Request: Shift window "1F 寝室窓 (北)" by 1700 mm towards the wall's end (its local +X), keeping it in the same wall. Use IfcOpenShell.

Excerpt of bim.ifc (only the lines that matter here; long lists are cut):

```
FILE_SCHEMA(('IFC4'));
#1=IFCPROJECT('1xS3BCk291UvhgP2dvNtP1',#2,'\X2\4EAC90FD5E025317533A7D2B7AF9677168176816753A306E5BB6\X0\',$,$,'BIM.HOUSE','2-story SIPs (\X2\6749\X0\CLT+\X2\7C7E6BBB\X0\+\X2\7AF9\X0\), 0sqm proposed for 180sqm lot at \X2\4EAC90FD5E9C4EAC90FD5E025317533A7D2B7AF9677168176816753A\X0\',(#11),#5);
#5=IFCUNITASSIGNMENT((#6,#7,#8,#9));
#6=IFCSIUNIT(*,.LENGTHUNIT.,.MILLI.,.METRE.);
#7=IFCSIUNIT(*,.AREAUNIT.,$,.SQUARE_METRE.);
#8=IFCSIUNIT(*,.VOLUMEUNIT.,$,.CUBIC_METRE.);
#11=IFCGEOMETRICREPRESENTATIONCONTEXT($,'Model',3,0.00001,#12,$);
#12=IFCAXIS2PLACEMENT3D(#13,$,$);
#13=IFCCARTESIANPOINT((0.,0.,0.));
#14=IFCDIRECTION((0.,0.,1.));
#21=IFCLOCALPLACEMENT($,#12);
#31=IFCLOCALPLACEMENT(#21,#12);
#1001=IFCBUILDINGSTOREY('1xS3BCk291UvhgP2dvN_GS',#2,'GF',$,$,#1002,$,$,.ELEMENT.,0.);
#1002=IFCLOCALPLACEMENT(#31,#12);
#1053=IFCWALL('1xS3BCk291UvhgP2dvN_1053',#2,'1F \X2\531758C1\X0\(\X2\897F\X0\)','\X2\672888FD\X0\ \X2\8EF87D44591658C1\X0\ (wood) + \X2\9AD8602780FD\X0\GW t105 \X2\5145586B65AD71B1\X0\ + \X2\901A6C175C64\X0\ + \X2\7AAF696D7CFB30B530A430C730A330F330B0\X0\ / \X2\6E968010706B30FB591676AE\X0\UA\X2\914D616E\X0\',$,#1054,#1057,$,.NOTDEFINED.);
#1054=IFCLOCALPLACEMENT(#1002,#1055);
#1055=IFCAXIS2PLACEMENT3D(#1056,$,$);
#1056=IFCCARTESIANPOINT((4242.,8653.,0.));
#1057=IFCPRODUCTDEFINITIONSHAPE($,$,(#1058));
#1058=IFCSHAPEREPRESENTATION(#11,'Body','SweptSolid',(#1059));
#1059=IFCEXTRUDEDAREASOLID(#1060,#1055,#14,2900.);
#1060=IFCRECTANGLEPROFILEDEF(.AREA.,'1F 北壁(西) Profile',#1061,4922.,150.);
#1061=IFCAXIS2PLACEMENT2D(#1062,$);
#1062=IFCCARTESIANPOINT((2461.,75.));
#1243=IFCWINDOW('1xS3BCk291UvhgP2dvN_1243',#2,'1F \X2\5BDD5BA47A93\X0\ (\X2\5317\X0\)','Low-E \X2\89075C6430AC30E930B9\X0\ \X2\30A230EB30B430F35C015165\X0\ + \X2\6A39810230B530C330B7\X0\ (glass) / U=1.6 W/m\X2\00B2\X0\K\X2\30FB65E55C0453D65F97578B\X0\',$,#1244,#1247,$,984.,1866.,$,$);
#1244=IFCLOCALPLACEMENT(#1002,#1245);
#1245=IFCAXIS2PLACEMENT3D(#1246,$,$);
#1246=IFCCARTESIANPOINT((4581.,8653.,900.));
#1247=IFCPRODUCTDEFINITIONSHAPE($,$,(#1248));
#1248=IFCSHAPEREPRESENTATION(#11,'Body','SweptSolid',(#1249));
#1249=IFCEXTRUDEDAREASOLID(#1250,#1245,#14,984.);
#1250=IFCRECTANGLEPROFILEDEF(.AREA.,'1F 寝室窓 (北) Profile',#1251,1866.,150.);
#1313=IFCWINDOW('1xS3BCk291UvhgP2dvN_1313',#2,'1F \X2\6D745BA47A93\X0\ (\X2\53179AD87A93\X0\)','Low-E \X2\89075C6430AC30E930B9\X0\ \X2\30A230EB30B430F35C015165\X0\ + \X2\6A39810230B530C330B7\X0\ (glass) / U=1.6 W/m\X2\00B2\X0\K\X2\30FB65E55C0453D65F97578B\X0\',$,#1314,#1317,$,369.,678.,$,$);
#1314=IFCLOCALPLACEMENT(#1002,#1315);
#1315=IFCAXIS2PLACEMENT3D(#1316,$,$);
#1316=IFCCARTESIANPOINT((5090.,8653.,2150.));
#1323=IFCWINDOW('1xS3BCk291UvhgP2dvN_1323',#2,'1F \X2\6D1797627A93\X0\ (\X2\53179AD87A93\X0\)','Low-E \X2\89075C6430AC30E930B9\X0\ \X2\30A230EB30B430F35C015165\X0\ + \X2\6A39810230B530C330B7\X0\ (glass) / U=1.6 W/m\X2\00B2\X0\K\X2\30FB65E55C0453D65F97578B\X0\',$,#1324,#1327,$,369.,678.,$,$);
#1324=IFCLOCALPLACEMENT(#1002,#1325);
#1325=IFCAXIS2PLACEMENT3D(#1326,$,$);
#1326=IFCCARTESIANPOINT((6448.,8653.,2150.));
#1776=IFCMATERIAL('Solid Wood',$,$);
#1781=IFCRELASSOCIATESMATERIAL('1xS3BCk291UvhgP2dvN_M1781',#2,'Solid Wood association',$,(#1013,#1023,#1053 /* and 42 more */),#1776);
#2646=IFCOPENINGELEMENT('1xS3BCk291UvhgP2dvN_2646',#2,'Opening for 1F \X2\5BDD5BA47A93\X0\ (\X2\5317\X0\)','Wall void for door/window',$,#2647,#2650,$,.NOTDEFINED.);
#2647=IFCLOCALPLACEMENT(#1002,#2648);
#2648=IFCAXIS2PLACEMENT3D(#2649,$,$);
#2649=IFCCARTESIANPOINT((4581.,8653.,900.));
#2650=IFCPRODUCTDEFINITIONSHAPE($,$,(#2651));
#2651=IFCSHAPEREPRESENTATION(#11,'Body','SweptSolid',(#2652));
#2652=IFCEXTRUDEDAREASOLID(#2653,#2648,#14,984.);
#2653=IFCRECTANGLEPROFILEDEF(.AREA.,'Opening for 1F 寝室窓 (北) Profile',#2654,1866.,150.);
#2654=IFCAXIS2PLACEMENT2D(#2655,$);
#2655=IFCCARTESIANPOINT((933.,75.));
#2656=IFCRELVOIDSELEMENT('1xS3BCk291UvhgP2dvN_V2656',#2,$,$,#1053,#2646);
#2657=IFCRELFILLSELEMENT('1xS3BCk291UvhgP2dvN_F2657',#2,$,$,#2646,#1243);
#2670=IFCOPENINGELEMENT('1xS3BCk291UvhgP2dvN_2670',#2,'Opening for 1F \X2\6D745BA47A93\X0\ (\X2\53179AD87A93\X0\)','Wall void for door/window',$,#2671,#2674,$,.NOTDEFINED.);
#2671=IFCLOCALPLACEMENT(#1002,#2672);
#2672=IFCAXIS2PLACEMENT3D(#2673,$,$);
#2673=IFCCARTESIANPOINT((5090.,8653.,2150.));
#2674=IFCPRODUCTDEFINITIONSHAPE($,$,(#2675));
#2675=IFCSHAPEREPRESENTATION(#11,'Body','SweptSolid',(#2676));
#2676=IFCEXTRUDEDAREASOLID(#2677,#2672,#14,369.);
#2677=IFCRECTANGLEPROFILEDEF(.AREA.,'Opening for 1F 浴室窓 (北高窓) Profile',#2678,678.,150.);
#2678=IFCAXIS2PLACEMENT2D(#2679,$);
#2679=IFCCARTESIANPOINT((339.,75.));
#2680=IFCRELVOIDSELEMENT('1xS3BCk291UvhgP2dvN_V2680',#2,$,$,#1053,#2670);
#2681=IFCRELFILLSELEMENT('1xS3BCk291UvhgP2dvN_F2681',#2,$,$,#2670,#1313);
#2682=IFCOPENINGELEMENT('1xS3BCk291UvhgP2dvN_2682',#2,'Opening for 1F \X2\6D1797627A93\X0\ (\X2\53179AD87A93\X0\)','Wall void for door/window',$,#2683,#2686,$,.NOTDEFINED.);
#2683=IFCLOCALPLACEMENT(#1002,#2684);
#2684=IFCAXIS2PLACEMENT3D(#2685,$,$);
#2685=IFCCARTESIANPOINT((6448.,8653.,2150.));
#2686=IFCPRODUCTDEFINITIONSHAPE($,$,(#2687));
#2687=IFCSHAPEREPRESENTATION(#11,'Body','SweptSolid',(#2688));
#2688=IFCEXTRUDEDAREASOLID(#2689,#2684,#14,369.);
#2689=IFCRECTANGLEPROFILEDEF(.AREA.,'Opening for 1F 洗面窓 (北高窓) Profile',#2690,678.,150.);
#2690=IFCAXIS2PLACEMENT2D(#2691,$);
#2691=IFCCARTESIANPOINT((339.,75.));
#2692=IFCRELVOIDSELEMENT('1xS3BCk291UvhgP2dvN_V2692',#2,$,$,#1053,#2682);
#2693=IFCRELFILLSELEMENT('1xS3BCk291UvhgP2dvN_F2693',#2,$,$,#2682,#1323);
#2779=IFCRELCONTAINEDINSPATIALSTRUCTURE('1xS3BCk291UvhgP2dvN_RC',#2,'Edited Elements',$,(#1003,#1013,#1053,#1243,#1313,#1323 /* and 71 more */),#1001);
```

```python
import ifcopenshell
import ifcopenshell.api.geometry
import ifcopenshell.util.placement
import ifcopenshell.util.unit

model = ifcopenshell.open("bim.ifc")
unit_scale = ifcopenshell.util.unit.calculate_unit_scale(model)

window = model.by_guid("1xS3BCk291UvhgP2dvN_1243")
opening = window.FillsVoids[0].RelatingOpeningElement
wall = opening.VoidsElements[0].RelatingBuildingElement

wall_matrix = ifcopenshell.util.placement.get_local_placement(wall.ObjectPlacement)
shift = wall_matrix[:3, 0] * 1.7 / unit_scale
before = ifcopenshell.util.placement.get_local_placement(window.ObjectPlacement)[:3, 3].copy()

# The window is not placed relative to its opening, so move both.
for product in (opening, window):
    matrix = ifcopenshell.util.placement.get_local_placement(product.ObjectPlacement)
    matrix[:3, 3] += shift
    ifcopenshell.api.geometry.edit_object_placement(model, product=product, matrix=matrix, is_si=False)

after = ifcopenshell.util.placement.get_local_placement(window.ObjectPlacement)[:3, 3]
print("window moved by", (after - before).round(3) + 0.0)

model.write("bim_rev.ifc")
```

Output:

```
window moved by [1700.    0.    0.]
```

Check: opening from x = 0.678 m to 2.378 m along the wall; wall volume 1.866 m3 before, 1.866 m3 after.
